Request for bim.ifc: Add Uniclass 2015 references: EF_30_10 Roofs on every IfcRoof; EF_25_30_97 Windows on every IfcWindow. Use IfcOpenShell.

First a look at what the model holds.

```python
import ifcopenshell

model = ifcopenshell.open("bim.ifc")
print(model.schema)
print("classifications:", [c.Name for c in model.by_type("IfcClassification")])
for ifc_class in ("IfcDoor", "IfcRoof", "IfcStair", "IfcWall", "IfcWindow"):
    print(ifc_class, len(model.by_type(ifc_class)))
```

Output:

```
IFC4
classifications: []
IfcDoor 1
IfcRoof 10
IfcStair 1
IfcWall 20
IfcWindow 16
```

```python
import ifcopenshell
import ifcopenshell.api.classification

model = ifcopenshell.open("bim.ifc")

system = ifcopenshell.api.classification.add_classification(model, classification="Uniclass 2015")

codes = {
    "IfcRoof": ("EF_30_10", "Roofs"),
    "IfcWindow": ("EF_25_30_97", "Windows"),
}
for ifc_class, (code, name) in codes.items():
    products = model.by_type(ifc_class)
    ifcopenshell.api.classification.add_reference(
        model, products=products, classification=system, identification=code, name=name
    )
    print(code, len(products))

model.write("bim_v2.ifc")
```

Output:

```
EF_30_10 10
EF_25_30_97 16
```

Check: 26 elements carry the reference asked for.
